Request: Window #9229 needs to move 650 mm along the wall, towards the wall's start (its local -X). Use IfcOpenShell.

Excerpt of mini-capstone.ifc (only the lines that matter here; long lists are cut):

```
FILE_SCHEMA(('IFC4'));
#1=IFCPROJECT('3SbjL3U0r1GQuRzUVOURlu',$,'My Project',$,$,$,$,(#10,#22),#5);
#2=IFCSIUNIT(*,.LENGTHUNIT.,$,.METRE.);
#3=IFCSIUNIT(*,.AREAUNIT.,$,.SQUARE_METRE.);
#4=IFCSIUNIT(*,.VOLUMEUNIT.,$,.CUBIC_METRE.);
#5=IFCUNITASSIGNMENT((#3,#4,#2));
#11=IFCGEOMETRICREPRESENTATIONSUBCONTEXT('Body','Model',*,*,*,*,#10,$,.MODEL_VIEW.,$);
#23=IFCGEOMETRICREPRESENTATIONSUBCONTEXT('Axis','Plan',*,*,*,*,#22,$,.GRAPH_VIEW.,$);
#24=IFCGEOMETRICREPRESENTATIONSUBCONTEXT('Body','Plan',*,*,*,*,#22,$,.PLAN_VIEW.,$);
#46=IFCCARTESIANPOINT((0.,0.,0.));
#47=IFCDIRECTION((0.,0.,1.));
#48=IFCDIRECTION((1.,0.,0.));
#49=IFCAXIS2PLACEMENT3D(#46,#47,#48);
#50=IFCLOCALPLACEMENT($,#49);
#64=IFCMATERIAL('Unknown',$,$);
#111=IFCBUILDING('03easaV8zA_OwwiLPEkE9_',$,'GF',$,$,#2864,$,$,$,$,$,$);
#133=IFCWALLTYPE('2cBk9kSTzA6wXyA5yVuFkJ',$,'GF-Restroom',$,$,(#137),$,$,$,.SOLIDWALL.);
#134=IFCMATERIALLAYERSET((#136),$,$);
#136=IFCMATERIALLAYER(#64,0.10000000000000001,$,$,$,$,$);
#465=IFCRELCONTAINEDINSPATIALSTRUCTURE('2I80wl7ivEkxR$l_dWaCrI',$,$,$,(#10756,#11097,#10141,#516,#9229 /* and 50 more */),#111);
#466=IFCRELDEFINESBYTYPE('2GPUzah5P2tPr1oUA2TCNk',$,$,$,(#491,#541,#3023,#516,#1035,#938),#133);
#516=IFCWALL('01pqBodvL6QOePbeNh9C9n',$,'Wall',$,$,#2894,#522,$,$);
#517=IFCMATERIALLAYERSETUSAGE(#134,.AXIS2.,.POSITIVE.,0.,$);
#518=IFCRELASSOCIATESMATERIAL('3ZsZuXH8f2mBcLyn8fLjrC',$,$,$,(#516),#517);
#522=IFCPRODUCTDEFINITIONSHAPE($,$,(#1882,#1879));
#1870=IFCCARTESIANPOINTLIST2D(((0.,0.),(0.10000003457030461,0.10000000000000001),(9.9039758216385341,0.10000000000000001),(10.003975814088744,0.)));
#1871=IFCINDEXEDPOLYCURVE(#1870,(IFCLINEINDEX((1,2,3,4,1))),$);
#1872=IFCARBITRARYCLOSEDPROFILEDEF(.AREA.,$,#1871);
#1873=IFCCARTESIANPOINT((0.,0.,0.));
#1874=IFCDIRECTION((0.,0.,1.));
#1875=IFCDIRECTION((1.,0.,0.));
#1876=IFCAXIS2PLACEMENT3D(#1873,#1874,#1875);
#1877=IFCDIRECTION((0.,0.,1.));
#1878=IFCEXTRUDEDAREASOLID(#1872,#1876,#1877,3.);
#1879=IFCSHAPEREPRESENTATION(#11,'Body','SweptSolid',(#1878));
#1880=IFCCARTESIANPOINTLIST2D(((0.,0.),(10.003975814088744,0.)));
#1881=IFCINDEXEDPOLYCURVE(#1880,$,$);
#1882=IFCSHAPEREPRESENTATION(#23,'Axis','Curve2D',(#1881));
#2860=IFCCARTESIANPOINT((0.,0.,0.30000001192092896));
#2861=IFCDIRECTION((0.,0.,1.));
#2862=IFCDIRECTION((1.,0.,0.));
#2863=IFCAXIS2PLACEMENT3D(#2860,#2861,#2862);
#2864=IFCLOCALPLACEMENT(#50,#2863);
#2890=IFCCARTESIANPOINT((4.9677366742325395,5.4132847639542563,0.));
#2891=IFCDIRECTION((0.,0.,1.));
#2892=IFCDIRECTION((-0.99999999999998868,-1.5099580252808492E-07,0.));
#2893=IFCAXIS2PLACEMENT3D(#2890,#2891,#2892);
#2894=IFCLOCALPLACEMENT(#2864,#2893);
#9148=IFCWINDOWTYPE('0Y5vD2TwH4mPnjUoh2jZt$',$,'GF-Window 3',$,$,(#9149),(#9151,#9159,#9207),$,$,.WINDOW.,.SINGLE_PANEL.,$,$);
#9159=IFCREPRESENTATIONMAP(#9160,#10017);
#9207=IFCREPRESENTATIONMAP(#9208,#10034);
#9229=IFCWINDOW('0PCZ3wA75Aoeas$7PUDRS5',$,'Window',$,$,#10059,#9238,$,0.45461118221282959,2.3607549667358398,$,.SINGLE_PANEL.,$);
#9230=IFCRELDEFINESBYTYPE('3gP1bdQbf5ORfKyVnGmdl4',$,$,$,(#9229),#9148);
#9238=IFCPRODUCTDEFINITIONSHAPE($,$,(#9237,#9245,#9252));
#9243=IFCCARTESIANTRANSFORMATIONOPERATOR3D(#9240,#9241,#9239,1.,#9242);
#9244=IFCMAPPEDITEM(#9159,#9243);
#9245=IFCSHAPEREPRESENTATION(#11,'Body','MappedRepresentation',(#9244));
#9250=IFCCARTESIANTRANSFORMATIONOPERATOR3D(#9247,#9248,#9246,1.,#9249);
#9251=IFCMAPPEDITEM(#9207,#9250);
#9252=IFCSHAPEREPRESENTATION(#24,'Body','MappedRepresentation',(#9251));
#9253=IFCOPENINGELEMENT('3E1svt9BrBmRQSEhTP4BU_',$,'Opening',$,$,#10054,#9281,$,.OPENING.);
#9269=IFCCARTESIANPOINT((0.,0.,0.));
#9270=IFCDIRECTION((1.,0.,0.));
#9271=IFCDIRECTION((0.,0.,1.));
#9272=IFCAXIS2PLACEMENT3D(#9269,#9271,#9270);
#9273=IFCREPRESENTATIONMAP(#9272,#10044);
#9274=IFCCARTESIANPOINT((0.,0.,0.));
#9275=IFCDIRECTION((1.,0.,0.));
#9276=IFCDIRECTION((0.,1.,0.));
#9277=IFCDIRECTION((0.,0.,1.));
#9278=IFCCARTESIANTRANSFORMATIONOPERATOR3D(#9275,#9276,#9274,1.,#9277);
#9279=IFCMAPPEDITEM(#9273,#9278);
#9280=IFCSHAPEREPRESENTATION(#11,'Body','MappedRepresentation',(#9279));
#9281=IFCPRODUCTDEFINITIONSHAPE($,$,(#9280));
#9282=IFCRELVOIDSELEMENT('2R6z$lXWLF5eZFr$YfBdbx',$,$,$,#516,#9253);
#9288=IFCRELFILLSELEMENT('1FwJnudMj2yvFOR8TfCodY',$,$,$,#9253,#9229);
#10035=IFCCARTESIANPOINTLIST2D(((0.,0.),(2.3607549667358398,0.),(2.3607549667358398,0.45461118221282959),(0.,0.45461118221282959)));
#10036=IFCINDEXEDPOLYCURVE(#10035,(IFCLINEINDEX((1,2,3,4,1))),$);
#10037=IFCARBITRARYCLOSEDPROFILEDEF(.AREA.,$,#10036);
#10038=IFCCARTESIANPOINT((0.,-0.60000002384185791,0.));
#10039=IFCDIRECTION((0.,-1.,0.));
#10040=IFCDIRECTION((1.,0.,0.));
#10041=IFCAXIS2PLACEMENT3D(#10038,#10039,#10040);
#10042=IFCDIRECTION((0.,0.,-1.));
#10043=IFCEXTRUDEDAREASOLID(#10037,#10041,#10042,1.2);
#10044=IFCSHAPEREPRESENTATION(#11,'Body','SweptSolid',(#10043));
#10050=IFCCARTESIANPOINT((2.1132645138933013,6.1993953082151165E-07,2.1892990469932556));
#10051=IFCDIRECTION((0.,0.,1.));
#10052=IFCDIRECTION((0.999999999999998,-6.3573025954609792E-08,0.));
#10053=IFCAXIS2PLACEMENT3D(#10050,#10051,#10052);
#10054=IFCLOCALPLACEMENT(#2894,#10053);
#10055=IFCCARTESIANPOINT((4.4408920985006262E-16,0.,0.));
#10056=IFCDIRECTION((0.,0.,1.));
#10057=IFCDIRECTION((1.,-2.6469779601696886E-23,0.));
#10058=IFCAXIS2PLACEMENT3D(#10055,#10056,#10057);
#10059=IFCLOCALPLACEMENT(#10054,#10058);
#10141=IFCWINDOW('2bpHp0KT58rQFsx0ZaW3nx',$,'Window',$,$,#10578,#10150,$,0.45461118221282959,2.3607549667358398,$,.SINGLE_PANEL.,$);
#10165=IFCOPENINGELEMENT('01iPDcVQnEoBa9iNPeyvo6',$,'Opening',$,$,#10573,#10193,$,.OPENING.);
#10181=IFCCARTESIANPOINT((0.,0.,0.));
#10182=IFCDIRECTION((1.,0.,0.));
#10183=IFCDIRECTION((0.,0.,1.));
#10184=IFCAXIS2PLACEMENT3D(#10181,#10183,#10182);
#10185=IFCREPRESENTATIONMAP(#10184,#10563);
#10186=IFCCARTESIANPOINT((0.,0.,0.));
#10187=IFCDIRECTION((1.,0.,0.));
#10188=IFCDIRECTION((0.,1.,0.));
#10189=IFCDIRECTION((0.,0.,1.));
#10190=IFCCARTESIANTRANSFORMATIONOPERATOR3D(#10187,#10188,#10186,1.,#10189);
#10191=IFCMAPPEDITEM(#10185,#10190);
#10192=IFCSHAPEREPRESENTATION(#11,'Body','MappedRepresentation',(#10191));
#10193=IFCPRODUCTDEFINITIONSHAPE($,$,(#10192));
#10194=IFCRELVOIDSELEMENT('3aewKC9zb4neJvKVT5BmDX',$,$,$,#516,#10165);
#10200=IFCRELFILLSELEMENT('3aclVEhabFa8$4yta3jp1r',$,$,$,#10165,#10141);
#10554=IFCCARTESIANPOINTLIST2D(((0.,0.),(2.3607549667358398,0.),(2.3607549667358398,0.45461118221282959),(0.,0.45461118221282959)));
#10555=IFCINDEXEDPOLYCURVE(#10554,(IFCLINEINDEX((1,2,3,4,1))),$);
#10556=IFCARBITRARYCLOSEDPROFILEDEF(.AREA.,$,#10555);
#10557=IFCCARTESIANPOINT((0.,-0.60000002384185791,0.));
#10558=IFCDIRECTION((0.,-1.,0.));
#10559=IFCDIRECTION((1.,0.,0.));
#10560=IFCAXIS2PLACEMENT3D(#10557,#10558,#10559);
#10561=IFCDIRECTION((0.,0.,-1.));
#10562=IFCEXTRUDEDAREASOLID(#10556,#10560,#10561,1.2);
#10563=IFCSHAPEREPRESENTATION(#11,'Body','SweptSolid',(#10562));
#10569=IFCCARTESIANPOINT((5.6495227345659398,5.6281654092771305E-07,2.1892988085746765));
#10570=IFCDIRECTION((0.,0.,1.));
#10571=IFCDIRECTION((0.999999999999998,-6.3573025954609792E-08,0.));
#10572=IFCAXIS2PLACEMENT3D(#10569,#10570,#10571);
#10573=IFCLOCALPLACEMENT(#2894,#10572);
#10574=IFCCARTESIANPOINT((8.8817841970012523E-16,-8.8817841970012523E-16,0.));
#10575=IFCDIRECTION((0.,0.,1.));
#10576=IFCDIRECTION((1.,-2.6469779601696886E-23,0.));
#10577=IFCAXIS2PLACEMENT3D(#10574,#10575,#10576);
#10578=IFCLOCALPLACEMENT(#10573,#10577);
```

```python
import ifcopenshell
import ifcopenshell.api.geometry
import ifcopenshell.util.placement
import ifcopenshell.util.unit

model = ifcopenshell.open("mini-capstone.ifc")
unit_scale = ifcopenshell.util.unit.calculate_unit_scale(model)

window = model.by_guid("0PCZ3wA75Aoeas$7PUDRS5")
opening = window.FillsVoids[0].RelatingOpeningElement
wall = opening.VoidsElements[0].RelatingBuildingElement

wall_matrix = ifcopenshell.util.placement.get_local_placement(wall.ObjectPlacement)
shift = wall_matrix[:3, 0] * -0.65 / unit_scale
before = ifcopenshell.util.placement.get_local_placement(window.ObjectPlacement)[:3, 3].copy()

# The window is placed relative to its opening, so it follows when the opening moves.
matrix = ifcopenshell.util.placement.get_local_placement(opening.ObjectPlacement)
matrix[:3, 3] += shift
ifcopenshell.api.geometry.edit_object_placement(
    model, product=opening, matrix=matrix, is_si=False, should_transform_children=True
)

after = ifcopenshell.util.placement.get_local_placement(window.ObjectPlacement)[:3, 3]
print("window moved by", (after - before).round(3) + 0.0)

model.write("mini-capstone-out.ifc")
```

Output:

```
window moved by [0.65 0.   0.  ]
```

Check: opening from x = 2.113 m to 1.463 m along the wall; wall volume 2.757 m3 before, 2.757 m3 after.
